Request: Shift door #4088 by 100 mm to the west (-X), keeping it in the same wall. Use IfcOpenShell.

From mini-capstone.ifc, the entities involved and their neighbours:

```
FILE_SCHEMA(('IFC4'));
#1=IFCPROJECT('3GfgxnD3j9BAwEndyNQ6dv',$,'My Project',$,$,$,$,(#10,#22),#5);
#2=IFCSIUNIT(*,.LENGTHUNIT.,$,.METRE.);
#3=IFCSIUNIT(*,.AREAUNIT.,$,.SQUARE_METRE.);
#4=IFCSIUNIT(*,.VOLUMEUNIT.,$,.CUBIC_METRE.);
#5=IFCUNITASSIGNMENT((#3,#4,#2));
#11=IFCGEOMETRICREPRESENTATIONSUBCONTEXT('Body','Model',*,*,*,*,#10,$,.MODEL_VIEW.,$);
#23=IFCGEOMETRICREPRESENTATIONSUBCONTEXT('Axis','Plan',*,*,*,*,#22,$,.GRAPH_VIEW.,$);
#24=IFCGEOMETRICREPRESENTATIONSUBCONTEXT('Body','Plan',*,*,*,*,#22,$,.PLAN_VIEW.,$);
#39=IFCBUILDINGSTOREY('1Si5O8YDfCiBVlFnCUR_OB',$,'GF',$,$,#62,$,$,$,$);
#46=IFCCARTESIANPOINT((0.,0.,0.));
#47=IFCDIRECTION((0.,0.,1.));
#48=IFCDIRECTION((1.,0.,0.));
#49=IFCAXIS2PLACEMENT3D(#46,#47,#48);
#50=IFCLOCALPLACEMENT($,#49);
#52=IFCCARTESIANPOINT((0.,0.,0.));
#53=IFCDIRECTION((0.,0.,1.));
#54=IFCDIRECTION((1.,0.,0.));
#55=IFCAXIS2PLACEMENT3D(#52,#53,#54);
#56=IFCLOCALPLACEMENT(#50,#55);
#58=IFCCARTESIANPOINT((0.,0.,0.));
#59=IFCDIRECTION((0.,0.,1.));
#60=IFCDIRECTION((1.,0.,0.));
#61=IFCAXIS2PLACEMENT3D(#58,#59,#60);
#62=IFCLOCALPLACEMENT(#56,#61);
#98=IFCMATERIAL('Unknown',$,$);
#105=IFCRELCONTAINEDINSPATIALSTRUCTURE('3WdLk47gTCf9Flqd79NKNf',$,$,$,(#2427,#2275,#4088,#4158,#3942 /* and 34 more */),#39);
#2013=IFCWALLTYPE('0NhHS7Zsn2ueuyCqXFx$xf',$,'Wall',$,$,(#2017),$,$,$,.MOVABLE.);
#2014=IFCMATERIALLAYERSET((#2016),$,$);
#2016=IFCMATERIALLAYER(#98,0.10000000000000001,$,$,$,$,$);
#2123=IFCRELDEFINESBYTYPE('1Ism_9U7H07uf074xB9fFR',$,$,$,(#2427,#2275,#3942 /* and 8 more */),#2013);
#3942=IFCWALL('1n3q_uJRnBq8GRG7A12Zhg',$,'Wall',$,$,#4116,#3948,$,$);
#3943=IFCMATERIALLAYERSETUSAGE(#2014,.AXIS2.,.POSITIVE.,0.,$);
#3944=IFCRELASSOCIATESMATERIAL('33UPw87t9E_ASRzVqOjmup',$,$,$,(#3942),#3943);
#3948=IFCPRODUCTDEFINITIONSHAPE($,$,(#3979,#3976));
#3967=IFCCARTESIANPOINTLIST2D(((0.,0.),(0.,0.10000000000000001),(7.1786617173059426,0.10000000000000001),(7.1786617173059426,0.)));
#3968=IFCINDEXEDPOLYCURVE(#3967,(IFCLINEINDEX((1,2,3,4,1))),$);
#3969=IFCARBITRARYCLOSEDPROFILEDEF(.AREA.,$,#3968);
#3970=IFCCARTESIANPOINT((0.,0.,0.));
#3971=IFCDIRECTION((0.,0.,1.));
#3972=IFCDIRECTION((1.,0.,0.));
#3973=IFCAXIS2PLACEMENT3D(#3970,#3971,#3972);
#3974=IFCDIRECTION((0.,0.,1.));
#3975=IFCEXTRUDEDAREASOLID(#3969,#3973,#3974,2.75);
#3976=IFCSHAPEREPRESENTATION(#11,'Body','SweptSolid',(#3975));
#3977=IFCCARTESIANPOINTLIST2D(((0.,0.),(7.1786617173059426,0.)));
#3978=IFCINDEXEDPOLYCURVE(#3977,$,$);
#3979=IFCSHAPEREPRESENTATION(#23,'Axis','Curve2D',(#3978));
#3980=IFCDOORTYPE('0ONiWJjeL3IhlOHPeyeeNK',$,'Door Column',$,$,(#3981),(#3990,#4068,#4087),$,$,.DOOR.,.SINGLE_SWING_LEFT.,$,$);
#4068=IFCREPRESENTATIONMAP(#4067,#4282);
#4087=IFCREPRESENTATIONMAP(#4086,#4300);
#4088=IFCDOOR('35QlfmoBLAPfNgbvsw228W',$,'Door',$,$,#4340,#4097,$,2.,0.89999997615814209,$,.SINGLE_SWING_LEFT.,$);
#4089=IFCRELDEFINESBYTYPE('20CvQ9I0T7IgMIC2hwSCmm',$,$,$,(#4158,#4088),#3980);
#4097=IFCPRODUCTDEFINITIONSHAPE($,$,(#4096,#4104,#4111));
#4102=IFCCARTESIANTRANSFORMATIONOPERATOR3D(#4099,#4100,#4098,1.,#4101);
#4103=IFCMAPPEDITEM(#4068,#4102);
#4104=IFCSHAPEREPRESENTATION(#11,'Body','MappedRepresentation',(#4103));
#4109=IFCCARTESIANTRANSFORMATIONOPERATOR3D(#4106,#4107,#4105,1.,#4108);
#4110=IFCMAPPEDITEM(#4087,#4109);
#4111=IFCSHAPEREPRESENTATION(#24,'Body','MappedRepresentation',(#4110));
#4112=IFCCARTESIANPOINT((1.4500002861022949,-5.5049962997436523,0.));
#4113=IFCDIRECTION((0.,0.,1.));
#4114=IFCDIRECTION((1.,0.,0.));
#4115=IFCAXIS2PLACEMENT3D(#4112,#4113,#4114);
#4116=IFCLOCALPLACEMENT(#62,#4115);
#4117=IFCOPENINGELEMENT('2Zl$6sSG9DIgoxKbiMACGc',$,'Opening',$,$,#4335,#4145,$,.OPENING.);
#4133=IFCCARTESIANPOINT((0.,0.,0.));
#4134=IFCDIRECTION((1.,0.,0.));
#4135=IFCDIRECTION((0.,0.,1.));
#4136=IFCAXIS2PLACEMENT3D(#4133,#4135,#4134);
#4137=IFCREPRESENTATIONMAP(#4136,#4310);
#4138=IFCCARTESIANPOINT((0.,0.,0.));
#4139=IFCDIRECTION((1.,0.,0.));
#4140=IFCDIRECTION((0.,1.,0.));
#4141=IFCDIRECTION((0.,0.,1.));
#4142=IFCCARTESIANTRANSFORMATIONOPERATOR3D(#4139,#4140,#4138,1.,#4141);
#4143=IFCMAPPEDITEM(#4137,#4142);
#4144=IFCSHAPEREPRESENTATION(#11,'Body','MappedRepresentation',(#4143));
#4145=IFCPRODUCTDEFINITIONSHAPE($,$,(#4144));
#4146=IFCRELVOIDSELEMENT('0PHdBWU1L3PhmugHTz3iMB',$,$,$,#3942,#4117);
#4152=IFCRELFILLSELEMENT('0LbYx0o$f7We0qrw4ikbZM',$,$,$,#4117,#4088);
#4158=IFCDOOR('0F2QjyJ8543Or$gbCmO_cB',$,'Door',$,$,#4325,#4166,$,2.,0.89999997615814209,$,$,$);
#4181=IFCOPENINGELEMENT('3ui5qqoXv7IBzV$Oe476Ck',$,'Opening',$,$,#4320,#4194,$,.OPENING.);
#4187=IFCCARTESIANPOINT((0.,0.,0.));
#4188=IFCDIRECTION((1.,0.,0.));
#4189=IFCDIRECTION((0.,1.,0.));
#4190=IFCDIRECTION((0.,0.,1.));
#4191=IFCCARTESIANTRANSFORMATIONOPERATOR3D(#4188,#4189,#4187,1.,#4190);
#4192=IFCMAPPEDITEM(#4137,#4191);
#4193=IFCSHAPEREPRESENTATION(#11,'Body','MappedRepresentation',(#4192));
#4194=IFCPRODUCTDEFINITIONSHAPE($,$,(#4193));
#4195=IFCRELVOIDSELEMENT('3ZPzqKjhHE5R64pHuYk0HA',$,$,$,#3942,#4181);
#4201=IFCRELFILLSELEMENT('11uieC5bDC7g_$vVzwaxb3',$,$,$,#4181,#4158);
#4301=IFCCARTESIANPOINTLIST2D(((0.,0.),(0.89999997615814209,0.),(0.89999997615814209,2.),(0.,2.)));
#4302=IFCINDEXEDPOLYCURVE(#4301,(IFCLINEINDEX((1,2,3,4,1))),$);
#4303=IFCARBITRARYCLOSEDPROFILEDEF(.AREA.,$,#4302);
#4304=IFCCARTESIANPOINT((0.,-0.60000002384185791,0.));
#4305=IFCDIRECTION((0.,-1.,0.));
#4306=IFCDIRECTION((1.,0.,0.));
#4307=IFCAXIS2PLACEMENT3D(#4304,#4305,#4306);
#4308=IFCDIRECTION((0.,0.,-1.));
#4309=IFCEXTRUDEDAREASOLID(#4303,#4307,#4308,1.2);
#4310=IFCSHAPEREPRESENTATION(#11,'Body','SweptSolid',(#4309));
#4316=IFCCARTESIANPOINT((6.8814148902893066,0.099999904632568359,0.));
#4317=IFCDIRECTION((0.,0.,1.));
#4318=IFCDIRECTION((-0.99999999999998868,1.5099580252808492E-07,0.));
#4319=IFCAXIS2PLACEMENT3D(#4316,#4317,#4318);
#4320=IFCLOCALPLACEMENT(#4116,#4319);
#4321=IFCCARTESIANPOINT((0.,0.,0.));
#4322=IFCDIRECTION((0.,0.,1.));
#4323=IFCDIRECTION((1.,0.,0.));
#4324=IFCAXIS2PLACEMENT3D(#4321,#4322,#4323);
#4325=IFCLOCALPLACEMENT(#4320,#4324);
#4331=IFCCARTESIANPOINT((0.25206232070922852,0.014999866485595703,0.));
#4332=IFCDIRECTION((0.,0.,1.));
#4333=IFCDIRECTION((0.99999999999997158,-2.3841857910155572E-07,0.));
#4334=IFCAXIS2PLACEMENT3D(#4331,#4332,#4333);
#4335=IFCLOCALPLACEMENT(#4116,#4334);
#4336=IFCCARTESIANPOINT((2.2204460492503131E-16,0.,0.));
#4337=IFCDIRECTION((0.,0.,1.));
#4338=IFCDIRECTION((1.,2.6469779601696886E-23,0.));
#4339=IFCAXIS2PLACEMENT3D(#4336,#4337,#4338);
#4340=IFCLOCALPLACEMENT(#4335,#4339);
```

```python
import ifcopenshell
import ifcopenshell.api.geometry
import ifcopenshell.util.placement
import ifcopenshell.util.unit

model = ifcopenshell.open("mini-capstone.ifc")
unit_scale = ifcopenshell.util.unit.calculate_unit_scale(model)

door = model.by_guid("35QlfmoBLAPfNgbvsw228W")
opening = door.FillsVoids[0].RelatingOpeningElement
wall = opening.VoidsElements[0].RelatingBuildingElement

wall_matrix = ifcopenshell.util.placement.get_local_placement(wall.ObjectPlacement)
shift = wall_matrix[:3, 0] * -0.1 / unit_scale
before = ifcopenshell.util.placement.get_local_placement(door.ObjectPlacement)[:3, 3].copy()

# The door is placed relative to its opening, so it follows when the opening moves.
matrix = ifcopenshell.util.placement.get_local_placement(opening.ObjectPlacement)
matrix[:3, 3] += shift
ifcopenshell.api.geometry.edit_object_placement(
    model, product=opening, matrix=matrix, is_si=False, should_transform_children=True
)

after = ifcopenshell.util.placement.get_local_placement(door.ObjectPlacement)[:3, 3]
print("door moved by", (after - before).round(3) + 0.0)

model.write("mini-capstone_v2.ifc")
```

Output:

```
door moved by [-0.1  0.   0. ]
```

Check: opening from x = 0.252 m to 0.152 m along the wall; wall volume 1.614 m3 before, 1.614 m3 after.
